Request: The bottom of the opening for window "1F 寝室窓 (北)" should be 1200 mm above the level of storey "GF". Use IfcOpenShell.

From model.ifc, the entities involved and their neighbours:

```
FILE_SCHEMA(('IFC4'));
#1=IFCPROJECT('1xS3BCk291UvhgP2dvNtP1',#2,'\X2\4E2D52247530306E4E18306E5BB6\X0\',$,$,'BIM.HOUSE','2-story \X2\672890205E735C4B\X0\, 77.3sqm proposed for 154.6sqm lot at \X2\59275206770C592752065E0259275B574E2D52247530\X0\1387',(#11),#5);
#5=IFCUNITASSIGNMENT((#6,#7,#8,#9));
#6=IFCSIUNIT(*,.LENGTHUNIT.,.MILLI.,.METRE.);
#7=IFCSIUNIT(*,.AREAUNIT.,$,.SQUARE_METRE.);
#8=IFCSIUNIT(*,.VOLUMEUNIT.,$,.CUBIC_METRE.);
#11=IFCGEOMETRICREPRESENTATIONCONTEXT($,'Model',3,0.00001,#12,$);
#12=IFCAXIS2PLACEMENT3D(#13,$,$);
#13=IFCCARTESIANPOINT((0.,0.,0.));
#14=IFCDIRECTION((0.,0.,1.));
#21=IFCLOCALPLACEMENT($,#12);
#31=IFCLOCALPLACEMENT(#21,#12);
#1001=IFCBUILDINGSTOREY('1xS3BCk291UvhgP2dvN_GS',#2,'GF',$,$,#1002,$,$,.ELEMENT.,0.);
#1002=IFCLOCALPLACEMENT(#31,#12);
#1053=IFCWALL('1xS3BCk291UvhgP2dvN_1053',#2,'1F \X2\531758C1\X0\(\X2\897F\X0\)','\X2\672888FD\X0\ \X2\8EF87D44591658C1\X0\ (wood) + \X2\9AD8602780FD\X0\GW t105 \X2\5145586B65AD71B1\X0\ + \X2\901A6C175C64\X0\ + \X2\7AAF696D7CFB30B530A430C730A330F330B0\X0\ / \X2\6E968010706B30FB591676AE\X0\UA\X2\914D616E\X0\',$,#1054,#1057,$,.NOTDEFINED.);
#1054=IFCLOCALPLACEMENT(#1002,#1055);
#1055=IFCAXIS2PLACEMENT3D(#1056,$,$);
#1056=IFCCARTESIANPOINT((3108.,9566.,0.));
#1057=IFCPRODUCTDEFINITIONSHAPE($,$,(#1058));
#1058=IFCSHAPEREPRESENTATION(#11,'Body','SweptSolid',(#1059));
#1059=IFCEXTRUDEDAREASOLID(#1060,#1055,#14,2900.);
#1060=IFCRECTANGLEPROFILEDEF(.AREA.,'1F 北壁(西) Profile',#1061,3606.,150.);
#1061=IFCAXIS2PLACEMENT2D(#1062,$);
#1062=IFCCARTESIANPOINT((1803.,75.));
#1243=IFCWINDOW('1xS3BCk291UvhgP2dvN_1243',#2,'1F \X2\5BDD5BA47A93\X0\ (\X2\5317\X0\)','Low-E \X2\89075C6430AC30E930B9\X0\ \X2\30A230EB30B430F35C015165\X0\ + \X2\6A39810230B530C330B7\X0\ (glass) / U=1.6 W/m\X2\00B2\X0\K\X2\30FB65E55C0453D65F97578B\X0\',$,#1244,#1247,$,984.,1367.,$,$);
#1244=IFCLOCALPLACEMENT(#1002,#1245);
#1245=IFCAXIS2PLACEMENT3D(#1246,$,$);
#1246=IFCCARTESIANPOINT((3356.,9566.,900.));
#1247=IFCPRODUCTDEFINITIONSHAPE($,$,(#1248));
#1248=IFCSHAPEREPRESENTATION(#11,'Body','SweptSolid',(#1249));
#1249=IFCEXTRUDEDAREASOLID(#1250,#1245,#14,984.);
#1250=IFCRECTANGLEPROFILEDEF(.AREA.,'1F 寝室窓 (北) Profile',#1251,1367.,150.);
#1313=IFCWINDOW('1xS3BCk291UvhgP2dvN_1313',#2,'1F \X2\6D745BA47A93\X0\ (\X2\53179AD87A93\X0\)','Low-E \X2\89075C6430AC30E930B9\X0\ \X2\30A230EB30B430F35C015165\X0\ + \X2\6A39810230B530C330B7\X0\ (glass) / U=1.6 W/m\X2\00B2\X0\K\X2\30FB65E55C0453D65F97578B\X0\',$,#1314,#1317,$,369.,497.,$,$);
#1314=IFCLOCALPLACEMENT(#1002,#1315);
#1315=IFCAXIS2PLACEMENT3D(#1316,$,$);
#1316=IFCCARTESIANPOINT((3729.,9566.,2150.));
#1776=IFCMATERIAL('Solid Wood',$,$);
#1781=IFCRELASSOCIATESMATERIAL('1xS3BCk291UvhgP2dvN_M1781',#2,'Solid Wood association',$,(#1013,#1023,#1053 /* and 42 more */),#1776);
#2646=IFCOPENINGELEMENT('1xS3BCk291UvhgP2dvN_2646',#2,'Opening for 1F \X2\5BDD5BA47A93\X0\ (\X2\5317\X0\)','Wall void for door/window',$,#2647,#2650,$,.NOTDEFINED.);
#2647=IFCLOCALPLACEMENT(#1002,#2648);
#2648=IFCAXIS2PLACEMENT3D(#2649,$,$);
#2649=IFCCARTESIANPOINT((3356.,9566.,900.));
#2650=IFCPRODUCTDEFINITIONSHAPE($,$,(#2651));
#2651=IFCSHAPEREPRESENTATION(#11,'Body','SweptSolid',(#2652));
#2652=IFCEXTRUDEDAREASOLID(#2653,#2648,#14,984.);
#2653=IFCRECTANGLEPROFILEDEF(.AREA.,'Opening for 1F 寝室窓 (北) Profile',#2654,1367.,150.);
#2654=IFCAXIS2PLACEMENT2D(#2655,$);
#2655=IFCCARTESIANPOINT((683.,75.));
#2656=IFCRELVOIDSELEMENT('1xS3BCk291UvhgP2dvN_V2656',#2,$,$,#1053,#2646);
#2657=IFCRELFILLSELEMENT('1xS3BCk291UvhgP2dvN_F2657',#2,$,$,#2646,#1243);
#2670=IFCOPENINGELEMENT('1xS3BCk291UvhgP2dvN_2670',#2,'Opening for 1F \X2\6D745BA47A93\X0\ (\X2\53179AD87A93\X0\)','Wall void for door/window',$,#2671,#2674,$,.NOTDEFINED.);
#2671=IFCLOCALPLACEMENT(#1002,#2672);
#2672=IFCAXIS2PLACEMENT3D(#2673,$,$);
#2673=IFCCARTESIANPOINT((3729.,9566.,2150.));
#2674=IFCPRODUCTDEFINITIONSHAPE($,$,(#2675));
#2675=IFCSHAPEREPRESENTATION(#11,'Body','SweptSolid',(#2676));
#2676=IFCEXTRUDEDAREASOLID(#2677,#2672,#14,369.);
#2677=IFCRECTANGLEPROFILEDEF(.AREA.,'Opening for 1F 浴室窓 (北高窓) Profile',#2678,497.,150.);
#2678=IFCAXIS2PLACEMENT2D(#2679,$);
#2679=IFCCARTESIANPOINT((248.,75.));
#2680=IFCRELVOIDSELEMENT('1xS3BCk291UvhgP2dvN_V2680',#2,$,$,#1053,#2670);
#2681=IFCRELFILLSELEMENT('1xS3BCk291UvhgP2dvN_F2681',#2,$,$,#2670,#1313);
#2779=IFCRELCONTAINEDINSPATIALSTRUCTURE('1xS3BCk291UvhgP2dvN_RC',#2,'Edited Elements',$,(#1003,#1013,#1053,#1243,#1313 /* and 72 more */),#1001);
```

```python
import numpy as np
import ifcopenshell
import ifcopenshell.api.geometry
import ifcopenshell.geom
import ifcopenshell.util.element
import ifcopenshell.util.placement
import ifcopenshell.util.shape
import ifcopenshell.util.unit

model = ifcopenshell.open("model.ifc")
unit_scale = ifcopenshell.util.unit.calculate_unit_scale(model)

window = model.by_guid("1xS3BCk291UvhgP2dvN_1243")
opening = window.FillsVoids[0].RelatingOpeningElement
storey = ifcopenshell.util.element.get_container(window, ifc_class="IfcBuildingStorey")
level = ifcopenshell.util.placement.get_local_placement(storey.ObjectPlacement)[2, 3]

# The opening's origin need not be at the sill, so measure its lowest point.
shape = ifcopenshell.geom.create_shape(ifcopenshell.geom.settings(), opening)
bottom = ifcopenshell.util.shape.get_shape_bottom_elevation(shape, shape.geometry) / unit_scale
dz = level + 1.2 / unit_scale - bottom

shift = np.array([0.0, 0.0, dz])
# The window is not placed relative to its opening, so move both.
for product in (opening, window):
    matrix = ifcopenshell.util.placement.get_local_placement(product.ObjectPlacement)
    matrix[:3, 3] += shift
    ifcopenshell.api.geometry.edit_object_placement(model, product=product, matrix=matrix, is_si=False)

print(f"moved by {dz * unit_scale:+.3f} m")

model.write("model_v2.ifc")
```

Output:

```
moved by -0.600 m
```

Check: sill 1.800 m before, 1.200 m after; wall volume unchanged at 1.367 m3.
